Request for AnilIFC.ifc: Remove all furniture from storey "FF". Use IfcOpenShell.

First a look at what the model holds.

```python
import ifcopenshell
import ifcopenshell.util.element

model = ifcopenshell.open("AnilIFC.ifc")
print(model.schema)
storey = next(s for s in model.by_type("IfcBuildingStorey") if s.Name == "FF")
furniture = [e for e in ifcopenshell.util.element.get_decomposition(storey) if e.is_a("IfcFurnishingElement")]
seen = {}
for e in furniture:
    element_type = ifcopenshell.util.element.get_type(e)
    name = element_type.Name if element_type not in (None, e) else None
    seen[name] = seen.get(name, 0) + 1
for name, count in sorted(seen.items(), key=str):
    print(count, "x", name)
```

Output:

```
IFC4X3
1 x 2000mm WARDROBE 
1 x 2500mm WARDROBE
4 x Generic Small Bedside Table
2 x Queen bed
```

```python
import ifcopenshell
import ifcopenshell.api.root
import ifcopenshell.util.element

model = ifcopenshell.open("AnilIFC.ifc")

storey = next(s for s in model.by_type("IfcBuildingStorey") if s.Name == "FF")
furniture = [e for e in ifcopenshell.util.element.get_decomposition(storey) if e.is_a("IfcFurnishingElement")]

for e in furniture:
    ifcopenshell.api.root.remove_product(model, product=e)
print(len(furniture), "removed")

model.write("AnilIFC_v2.ifc")
```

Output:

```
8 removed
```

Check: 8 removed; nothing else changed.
